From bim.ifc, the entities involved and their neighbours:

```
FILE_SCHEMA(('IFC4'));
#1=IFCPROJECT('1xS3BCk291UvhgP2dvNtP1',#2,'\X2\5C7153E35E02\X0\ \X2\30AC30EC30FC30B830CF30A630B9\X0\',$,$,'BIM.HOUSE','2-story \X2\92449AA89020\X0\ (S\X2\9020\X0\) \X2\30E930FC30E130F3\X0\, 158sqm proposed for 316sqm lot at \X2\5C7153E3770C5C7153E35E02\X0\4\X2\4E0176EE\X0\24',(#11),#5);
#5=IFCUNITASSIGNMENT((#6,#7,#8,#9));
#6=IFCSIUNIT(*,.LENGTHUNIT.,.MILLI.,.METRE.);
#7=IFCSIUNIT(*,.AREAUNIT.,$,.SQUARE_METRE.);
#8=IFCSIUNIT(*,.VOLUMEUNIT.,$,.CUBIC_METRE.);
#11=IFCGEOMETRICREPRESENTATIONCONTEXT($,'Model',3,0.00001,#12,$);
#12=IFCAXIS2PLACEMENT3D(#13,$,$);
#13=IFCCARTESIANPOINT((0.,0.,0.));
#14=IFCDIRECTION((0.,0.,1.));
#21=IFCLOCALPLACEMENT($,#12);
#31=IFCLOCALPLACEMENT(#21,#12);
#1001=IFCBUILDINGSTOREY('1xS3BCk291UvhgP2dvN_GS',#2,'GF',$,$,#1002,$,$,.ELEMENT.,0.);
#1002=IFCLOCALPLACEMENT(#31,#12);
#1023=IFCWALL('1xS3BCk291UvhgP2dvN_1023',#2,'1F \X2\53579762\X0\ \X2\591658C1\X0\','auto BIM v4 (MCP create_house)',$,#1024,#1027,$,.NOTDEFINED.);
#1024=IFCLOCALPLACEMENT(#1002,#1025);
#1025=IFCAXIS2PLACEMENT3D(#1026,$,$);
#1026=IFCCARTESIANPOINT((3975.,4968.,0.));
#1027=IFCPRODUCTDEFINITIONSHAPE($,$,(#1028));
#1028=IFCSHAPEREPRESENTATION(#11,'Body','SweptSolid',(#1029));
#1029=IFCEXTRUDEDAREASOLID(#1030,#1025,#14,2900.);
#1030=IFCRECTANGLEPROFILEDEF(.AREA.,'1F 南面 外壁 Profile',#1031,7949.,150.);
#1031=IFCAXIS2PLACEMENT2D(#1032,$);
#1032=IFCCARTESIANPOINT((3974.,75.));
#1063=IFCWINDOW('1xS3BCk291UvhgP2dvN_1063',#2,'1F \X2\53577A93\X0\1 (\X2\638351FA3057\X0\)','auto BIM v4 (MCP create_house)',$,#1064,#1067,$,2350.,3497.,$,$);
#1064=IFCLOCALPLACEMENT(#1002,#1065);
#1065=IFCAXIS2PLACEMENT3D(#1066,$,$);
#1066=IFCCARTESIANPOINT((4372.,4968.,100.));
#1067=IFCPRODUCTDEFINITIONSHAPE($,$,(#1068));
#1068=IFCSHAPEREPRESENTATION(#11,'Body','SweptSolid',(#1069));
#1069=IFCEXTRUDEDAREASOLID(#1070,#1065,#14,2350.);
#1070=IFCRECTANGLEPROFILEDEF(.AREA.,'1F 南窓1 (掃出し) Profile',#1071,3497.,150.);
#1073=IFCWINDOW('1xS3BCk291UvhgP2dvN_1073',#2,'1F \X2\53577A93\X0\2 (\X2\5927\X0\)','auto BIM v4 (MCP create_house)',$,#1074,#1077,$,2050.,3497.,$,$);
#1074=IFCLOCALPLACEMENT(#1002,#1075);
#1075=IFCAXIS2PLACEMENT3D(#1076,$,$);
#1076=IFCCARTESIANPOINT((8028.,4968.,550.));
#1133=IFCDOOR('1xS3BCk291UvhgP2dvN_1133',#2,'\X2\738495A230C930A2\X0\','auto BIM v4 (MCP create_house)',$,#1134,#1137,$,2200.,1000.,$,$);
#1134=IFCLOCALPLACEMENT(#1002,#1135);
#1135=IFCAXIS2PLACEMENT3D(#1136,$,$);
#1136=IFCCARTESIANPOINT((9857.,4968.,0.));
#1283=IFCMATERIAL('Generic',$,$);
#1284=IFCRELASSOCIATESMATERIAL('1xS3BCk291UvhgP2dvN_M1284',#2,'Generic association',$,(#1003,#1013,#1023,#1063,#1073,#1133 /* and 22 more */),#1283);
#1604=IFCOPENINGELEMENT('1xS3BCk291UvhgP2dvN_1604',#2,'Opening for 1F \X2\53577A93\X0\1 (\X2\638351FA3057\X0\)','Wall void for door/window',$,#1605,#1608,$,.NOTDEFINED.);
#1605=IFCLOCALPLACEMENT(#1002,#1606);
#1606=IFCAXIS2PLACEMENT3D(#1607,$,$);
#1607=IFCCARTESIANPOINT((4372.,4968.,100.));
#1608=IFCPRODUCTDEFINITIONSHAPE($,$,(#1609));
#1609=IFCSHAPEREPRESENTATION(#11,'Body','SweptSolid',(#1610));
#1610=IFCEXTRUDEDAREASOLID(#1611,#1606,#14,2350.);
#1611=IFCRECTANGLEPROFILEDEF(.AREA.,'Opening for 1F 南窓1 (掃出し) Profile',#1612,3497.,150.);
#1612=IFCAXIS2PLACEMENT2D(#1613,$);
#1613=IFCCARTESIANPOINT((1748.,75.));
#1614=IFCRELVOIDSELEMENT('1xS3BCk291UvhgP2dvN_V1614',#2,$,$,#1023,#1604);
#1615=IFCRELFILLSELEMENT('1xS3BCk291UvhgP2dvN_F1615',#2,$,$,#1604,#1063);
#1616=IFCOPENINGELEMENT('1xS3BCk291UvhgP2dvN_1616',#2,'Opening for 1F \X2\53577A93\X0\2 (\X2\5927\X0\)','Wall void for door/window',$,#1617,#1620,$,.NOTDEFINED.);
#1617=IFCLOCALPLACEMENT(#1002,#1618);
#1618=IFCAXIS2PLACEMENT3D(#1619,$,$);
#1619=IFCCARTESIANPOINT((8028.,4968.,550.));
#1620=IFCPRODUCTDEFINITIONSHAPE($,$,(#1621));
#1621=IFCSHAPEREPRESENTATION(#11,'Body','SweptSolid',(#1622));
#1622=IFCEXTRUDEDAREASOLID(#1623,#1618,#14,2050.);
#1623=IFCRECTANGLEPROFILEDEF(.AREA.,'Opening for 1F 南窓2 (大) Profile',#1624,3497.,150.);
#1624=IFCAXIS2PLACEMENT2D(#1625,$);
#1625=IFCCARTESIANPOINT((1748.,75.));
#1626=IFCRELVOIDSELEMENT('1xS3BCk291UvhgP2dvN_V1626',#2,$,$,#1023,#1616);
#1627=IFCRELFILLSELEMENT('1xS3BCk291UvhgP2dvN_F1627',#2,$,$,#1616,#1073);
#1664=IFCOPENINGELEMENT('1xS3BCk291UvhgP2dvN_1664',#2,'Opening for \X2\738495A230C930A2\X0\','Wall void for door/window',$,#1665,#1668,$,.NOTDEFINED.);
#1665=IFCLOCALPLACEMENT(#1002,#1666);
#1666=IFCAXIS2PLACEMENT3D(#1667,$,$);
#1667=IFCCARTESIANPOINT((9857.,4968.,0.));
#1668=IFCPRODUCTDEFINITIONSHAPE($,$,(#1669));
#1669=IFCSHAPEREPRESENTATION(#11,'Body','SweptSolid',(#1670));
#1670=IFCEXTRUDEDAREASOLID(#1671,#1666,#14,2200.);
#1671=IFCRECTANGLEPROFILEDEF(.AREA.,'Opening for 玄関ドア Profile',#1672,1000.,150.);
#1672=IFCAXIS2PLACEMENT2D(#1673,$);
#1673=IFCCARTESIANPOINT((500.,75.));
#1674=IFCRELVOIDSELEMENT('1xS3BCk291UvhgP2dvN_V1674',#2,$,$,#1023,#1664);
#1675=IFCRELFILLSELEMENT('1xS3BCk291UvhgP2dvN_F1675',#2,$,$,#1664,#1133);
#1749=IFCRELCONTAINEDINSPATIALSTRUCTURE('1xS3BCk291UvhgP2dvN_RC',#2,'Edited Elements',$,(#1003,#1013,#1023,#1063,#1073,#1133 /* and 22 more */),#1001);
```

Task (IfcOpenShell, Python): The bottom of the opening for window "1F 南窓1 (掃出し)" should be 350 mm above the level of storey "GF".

```python
import numpy as np
import ifcopenshell
import ifcopenshell.api.geometry
import ifcopenshell.geom
import ifcopenshell.util.element
import ifcopenshell.util.placement
import ifcopenshell.util.shape
import ifcopenshell.util.unit

model = ifcopenshell.open("bim.ifc")
unit_scale = ifcopenshell.util.unit.calculate_unit_scale(model)

window = model.by_guid("1xS3BCk291UvhgP2dvN_1063")
opening = window.FillsVoids[0].RelatingOpeningElement
storey = ifcopenshell.util.element.get_container(window, ifc_class="IfcBuildingStorey")
level = ifcopenshell.util.placement.get_local_placement(storey.ObjectPlacement)[2, 3]

# The opening's origin need not be at the sill, so measure its lowest point.
shape = ifcopenshell.geom.create_shape(ifcopenshell.geom.settings(), opening)
bottom = ifcopenshell.util.shape.get_shape_bottom_elevation(shape, shape.geometry) / unit_scale
dz = level + 0.35 / unit_scale - bottom

shift = np.array([0.0, 0.0, dz])
# The window is not placed relative to its opening, so move both.
for product in (opening, window):
    matrix = ifcopenshell.util.placement.get_local_placement(product.ObjectPlacement)
    matrix[:3, 3] += shift
    ifcopenshell.api.geometry.edit_object_placement(model, product=product, matrix=matrix, is_si=False)

print(f"moved by {dz * unit_scale:+.3f} m")

model.write("bim_edited.ifc")
```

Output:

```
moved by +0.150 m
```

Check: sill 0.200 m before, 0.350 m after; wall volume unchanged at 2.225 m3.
